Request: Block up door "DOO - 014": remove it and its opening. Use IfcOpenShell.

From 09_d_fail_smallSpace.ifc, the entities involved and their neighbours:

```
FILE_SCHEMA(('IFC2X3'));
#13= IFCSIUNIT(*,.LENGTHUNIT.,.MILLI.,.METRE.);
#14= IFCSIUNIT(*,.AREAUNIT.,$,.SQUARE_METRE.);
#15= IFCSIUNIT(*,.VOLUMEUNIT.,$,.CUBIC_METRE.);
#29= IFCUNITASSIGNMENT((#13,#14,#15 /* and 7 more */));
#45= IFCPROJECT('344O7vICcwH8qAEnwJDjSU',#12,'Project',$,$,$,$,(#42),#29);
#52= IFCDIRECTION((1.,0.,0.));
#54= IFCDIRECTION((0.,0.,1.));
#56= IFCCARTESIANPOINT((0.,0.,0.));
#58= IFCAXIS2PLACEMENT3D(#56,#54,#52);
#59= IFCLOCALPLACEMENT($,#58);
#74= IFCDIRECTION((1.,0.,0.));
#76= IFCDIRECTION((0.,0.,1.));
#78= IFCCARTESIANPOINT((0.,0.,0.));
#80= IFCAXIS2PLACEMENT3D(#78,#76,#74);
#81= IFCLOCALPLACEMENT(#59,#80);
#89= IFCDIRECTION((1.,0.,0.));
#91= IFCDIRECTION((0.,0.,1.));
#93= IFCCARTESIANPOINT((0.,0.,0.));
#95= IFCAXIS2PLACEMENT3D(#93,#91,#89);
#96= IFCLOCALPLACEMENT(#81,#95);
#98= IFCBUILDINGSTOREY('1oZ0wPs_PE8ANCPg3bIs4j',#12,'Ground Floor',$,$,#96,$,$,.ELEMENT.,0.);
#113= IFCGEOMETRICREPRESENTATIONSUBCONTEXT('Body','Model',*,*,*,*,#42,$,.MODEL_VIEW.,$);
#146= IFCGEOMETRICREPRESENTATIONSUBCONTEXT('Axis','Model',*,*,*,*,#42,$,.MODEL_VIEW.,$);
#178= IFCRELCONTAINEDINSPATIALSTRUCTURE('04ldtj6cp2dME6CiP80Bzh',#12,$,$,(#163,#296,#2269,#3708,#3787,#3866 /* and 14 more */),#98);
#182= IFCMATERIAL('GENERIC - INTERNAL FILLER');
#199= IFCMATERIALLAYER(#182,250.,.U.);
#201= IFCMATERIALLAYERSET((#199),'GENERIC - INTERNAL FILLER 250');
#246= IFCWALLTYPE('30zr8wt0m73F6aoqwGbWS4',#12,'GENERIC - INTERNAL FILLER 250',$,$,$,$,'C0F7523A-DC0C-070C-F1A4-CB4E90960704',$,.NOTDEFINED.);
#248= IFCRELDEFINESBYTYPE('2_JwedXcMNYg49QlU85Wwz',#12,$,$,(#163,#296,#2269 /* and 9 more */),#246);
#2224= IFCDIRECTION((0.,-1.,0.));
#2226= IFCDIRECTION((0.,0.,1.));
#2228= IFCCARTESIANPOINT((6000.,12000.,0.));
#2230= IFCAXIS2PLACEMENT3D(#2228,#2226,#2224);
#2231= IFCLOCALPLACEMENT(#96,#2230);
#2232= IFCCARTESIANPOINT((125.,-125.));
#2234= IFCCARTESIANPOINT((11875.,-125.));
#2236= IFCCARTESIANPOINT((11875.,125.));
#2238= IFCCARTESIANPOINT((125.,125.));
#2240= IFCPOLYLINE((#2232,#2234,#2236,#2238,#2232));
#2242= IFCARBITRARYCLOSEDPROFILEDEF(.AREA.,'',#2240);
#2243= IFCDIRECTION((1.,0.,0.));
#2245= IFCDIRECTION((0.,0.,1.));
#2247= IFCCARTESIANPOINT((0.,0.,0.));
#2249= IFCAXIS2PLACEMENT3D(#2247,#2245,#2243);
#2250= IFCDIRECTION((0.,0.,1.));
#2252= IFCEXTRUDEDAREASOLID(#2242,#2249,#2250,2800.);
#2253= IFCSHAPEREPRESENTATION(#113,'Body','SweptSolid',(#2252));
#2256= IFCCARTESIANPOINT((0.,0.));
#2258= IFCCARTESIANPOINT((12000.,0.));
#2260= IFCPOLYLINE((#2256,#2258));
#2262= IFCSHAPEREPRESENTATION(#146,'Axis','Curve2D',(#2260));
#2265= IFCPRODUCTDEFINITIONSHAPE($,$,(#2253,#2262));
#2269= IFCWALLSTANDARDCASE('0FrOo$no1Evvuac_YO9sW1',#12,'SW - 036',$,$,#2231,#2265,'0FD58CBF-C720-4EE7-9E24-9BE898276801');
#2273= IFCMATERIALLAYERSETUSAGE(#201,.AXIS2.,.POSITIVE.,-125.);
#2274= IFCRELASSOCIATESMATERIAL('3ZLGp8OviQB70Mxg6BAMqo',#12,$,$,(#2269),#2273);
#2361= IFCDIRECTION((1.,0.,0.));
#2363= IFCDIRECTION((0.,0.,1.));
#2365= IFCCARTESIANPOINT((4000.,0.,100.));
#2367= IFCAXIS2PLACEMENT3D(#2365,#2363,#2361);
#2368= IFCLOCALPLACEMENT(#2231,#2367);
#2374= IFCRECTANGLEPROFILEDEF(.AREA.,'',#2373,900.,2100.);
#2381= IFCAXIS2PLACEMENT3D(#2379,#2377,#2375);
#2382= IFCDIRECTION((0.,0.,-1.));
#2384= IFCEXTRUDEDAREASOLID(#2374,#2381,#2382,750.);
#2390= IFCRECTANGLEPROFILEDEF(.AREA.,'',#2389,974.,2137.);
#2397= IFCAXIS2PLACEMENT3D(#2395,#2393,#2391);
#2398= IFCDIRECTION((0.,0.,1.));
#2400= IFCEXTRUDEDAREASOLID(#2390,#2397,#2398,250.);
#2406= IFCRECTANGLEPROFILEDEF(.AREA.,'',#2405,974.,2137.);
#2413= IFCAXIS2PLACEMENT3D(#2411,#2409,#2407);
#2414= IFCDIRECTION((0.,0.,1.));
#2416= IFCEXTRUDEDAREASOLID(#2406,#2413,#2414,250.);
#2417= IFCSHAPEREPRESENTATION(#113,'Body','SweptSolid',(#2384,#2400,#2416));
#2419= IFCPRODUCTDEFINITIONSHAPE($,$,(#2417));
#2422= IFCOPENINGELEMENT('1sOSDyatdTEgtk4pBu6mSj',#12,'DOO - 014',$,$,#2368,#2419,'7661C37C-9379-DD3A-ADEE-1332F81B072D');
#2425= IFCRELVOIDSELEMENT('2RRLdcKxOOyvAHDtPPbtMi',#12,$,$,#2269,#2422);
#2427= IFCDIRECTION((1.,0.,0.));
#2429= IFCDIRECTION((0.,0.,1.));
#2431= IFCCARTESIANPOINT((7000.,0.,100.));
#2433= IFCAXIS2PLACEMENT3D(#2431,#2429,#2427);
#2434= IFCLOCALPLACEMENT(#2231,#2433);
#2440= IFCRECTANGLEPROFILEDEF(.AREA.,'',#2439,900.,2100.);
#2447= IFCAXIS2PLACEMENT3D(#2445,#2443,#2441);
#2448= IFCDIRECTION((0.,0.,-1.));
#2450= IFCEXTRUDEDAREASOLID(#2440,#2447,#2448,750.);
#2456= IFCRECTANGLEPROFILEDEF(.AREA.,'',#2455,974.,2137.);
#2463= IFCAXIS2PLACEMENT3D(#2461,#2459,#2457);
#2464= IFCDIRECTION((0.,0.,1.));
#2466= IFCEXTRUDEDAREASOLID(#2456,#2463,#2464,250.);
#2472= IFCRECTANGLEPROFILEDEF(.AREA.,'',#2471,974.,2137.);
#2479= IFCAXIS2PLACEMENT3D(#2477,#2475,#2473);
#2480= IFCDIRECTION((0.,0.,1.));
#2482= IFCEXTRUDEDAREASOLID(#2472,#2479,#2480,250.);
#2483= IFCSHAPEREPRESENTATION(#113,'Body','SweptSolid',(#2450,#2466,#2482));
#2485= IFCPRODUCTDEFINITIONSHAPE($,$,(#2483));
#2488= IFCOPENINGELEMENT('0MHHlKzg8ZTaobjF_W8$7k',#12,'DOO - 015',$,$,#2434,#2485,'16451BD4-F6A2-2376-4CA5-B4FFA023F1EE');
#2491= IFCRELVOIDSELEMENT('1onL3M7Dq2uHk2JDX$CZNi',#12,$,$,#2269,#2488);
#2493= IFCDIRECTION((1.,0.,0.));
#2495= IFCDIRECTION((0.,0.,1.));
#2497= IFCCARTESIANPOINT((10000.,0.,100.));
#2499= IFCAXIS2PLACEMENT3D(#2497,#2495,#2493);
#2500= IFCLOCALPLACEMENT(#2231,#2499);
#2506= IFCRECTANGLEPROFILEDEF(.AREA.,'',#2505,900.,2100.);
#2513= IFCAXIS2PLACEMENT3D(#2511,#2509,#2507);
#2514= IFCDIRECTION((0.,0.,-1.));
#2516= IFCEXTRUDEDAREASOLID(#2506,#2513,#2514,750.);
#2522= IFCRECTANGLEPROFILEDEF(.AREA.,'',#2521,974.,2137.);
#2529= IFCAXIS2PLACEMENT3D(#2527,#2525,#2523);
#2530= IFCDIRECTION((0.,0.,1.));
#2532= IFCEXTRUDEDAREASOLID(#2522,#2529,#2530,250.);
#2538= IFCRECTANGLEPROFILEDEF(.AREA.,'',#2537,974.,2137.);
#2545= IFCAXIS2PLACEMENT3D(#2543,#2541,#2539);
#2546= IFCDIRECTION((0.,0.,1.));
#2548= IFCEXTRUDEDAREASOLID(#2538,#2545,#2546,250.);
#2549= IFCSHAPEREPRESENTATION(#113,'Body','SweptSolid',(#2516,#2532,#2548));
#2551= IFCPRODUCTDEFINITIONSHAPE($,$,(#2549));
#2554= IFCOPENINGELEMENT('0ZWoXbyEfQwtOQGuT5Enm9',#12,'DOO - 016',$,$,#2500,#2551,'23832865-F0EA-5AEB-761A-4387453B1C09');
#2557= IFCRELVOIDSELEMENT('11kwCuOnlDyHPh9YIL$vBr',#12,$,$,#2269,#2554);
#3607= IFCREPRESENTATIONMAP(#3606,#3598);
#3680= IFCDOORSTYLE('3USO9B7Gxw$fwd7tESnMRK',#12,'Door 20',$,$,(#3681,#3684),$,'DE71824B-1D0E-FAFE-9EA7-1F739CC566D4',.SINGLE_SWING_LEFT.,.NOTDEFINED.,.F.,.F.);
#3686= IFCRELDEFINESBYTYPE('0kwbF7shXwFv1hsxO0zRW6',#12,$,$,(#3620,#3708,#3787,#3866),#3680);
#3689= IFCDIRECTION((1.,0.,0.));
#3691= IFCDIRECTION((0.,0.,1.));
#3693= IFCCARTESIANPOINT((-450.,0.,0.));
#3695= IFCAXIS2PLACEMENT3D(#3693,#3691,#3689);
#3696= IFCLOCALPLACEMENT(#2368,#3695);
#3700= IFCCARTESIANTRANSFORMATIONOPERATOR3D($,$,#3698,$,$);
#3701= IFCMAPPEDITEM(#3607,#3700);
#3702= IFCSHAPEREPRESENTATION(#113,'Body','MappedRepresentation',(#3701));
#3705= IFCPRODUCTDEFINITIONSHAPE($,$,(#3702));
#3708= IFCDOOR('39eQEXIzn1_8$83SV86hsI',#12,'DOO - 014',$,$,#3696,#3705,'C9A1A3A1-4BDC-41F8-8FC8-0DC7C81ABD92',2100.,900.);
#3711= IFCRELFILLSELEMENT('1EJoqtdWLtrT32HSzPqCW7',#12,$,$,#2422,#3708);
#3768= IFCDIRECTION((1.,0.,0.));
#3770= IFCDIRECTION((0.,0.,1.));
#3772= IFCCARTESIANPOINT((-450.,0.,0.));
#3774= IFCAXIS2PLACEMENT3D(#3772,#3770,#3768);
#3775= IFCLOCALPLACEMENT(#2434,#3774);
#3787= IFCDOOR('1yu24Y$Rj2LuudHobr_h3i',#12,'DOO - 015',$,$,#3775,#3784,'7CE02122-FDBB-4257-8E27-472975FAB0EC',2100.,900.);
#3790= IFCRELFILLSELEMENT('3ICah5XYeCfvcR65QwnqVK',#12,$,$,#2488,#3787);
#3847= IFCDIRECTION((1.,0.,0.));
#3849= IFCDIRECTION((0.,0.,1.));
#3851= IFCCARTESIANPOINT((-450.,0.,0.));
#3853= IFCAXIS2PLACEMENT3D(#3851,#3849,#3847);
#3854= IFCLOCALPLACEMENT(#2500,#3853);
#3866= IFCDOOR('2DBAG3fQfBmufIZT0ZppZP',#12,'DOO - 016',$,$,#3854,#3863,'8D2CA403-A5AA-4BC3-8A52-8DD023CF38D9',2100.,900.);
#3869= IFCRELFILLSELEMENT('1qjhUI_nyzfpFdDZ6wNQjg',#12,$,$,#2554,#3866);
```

```python
import ifcopenshell
import ifcopenshell.api.feature
import ifcopenshell.api.root
import ifcopenshell.geom
import ifcopenshell.util.shape

model = ifcopenshell.open("09_d_fail_smallSpace.ifc")
settings = ifcopenshell.geom.settings()


def volume(element):
    """Net volume in cubic metres, openings subtracted."""
    shape = ifcopenshell.geom.create_shape(settings, element)
    return ifcopenshell.util.shape.get_volume(shape.geometry)


door = model.by_guid("39eQEXIzn1_8$83SV86hsI")
opening = door.FillsVoids[0].RelatingOpeningElement
wall = opening.VoidsElements[0].RelatingBuildingElement
before = volume(wall)

ifcopenshell.api.root.remove_product(model, product=door)
ifcopenshell.api.feature.remove_feature(model, feature=opening)

after = volume(wall)

print(f"wall volume {before:.3f} -> {after:.3f} m3")

model.write("09_d_fail_smallSpace_rev.ifc")
```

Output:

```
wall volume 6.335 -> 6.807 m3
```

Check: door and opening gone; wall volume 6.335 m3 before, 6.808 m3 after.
